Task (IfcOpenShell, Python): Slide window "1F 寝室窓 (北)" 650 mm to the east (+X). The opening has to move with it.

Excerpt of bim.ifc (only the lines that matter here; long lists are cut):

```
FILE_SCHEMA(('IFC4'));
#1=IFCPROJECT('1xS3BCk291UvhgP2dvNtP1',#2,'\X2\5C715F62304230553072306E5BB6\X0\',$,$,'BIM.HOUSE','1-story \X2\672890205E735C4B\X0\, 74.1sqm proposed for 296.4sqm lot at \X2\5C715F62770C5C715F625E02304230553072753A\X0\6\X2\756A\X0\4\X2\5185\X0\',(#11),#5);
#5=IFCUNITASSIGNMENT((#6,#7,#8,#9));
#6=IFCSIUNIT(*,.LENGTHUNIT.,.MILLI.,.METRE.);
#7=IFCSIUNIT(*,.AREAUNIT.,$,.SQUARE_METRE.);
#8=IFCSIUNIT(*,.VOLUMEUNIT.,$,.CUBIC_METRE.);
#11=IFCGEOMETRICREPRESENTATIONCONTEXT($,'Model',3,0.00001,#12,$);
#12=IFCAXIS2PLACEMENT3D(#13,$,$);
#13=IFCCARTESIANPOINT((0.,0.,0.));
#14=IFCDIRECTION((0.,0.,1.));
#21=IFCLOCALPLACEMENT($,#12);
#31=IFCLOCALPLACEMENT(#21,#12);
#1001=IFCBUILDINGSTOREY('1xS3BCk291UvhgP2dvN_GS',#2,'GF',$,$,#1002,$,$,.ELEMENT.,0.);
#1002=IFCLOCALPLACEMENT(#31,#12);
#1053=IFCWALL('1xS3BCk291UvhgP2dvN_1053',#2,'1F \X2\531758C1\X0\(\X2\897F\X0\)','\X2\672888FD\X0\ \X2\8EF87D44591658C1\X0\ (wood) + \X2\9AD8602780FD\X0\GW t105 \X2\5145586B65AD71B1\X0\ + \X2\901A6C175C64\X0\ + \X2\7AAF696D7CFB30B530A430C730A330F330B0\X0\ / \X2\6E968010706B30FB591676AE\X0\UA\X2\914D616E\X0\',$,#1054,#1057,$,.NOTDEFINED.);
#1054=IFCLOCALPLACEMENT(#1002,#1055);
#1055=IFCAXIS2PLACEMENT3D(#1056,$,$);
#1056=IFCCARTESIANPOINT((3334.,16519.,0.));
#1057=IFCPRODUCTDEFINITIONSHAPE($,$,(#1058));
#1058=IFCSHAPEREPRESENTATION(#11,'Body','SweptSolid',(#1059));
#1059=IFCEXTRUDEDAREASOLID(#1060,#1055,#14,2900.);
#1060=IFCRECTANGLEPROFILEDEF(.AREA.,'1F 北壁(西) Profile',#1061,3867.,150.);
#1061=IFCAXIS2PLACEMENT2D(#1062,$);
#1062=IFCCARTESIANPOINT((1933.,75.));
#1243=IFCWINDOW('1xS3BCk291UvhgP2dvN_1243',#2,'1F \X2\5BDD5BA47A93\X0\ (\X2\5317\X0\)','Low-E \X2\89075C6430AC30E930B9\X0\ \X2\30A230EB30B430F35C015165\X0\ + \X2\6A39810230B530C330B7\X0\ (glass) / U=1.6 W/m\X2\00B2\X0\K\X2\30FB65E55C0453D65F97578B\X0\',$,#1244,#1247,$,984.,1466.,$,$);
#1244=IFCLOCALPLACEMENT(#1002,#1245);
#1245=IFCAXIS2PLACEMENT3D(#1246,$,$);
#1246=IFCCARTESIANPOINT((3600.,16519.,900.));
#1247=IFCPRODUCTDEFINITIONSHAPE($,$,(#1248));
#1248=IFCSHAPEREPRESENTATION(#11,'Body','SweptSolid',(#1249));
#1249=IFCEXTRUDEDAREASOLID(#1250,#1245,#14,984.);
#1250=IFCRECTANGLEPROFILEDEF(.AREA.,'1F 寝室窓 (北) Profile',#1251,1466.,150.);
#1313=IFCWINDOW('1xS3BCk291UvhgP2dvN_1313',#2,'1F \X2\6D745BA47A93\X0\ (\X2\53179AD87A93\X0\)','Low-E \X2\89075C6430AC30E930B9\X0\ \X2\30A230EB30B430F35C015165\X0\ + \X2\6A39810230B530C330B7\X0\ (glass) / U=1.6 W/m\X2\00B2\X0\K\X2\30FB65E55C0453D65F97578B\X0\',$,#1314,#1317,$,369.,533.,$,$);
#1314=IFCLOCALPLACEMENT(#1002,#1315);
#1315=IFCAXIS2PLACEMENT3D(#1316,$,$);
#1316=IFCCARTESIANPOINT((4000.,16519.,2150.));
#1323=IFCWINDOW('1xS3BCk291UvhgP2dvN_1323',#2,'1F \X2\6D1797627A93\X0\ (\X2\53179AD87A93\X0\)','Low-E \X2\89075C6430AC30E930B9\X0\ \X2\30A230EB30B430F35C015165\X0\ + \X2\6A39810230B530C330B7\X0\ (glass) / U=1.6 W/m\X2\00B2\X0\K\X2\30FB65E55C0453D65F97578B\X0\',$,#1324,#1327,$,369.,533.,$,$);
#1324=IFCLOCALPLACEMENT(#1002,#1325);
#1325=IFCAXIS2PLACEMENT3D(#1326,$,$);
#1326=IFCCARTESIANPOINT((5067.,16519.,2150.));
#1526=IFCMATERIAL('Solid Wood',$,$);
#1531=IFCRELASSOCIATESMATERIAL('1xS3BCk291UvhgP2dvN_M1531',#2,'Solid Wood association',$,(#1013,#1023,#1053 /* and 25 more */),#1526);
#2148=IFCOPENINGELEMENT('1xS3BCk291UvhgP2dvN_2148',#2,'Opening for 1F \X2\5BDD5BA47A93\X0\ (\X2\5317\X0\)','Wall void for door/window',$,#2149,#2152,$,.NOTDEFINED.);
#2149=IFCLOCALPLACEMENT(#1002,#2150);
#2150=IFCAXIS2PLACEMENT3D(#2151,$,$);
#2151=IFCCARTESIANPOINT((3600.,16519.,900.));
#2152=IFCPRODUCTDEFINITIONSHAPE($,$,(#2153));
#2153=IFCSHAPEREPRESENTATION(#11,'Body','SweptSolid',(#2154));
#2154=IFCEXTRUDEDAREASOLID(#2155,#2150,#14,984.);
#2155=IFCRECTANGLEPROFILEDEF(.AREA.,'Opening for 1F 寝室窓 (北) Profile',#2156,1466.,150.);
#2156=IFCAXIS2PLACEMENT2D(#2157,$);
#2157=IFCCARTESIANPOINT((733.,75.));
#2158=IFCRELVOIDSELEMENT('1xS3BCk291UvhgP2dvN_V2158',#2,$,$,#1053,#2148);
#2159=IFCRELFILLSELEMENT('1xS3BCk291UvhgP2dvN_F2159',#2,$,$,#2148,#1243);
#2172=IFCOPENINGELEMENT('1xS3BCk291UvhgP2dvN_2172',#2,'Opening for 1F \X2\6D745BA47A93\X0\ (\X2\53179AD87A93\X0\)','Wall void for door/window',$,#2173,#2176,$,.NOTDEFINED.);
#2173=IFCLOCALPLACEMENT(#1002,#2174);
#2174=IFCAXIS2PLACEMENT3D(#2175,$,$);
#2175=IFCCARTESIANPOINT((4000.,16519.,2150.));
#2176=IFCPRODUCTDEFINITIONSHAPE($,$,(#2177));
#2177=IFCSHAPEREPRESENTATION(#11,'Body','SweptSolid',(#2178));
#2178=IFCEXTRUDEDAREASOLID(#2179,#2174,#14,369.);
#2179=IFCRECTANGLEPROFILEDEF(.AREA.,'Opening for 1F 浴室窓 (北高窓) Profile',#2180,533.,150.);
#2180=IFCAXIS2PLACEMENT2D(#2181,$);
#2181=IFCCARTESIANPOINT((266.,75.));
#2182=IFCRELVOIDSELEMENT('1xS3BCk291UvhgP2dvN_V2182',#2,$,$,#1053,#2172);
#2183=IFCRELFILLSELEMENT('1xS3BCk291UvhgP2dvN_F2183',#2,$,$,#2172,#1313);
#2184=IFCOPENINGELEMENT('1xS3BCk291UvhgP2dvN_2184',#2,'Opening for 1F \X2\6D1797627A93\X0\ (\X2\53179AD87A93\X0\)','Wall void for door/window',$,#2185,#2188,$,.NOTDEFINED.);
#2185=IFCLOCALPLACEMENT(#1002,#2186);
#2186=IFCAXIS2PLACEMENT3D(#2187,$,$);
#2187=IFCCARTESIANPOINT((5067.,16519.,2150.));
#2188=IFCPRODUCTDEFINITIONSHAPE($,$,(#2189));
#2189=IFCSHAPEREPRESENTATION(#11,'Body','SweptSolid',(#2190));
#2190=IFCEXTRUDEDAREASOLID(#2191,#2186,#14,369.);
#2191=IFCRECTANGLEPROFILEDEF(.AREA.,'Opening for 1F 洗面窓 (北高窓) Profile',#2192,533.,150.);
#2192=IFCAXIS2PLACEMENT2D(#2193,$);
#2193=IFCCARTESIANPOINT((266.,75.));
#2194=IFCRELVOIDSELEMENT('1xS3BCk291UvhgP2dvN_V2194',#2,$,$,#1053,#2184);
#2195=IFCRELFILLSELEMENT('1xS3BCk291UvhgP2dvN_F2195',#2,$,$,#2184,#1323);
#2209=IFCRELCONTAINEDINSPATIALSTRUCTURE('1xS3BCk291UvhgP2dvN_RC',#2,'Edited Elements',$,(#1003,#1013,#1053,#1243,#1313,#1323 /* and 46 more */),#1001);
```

```python
import ifcopenshell
import ifcopenshell.api.geometry
import ifcopenshell.util.placement
import ifcopenshell.util.unit

model = ifcopenshell.open("bim.ifc")
unit_scale = ifcopenshell.util.unit.calculate_unit_scale(model)

window = model.by_guid("1xS3BCk291UvhgP2dvN_1243")
opening = window.FillsVoids[0].RelatingOpeningElement
wall = opening.VoidsElements[0].RelatingBuildingElement

wall_matrix = ifcopenshell.util.placement.get_local_placement(wall.ObjectPlacement)
shift = wall_matrix[:3, 0] * 0.65 / unit_scale
before = ifcopenshell.util.placement.get_local_placement(window.ObjectPlacement)[:3, 3].copy()

# The window is not placed relative to its opening, so move both.
for product in (opening, window):
    matrix = ifcopenshell.util.placement.get_local_placement(product.ObjectPlacement)
    matrix[:3, 3] += shift
    ifcopenshell.api.geometry.edit_object_placement(model, product=product, matrix=matrix, is_si=False)

after = ifcopenshell.util.placement.get_local_placement(window.ObjectPlacement)[:3, 3]
print("window moved by", (after - before).round(3) + 0.0)

model.write("bim_edited.ifc")
```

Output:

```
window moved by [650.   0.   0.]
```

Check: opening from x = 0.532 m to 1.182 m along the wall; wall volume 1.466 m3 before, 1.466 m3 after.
